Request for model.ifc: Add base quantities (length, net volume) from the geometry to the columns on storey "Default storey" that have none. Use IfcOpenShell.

First a look at what the model holds.

```python
import ifcopenshell
import ifcopenshell.util.element
import ifcopenshell.util.unit

model = ifcopenshell.open("model.ifc")
print(model.schema)
for unit_type in ("LENGTHUNIT", "AREAUNIT", "VOLUMEUNIT"):
    print(unit_type, ifcopenshell.util.unit.calculate_unit_scale(model, unit_type))
storey = next(s for s in model.by_type("IfcBuildingStorey") if s.Name == "Default storey")
columns = [e for e in ifcopenshell.util.element.get_decomposition(storey) if e.is_a("IfcColumn")]
for e in sorted(columns, key=lambda e: e.id()):
    print(e.id(), e.is_a(), e.Name, list(ifcopenshell.util.element.get_psets(e, qtos_only=True)), sep=" | ")
```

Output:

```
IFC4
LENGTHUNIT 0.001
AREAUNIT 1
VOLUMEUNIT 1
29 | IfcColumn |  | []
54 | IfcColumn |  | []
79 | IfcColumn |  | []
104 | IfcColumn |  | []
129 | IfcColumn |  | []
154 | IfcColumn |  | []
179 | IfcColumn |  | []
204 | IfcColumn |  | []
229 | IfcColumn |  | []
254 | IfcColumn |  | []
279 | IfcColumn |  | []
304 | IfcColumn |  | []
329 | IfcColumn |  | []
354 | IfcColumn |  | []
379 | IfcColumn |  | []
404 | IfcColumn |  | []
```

```python
import ifcopenshell
import ifcopenshell.api.pset
import ifcopenshell.geom
import ifcopenshell.util.element
import ifcopenshell.util.shape
import ifcopenshell.util.unit

model = ifcopenshell.open("model.ifc")
unit_scale = ifcopenshell.util.unit.calculate_unit_scale(model)
volume_scale = ifcopenshell.util.unit.calculate_unit_scale(model, "VOLUMEUNIT")
settings = ifcopenshell.geom.settings()

storey = next(s for s in model.by_type("IfcBuildingStorey") if s.Name == "Default storey")
columns = [e for e in ifcopenshell.util.element.get_decomposition(storey) if e.is_a("IfcColumn")]

for e in sorted(columns, key=lambda e: e.id()):
    if ifcopenshell.util.element.get_psets(e, qtos_only=True, should_inherit=False):
        continue
    # Geometry comes back in metres, in the element's own axes.
    shape = ifcopenshell.geom.create_shape(settings, e)
    values = {
        "Length": ifcopenshell.util.shape.get_z(shape.geometry) / unit_scale,
        "NetVolume": ifcopenshell.util.shape.get_volume(shape.geometry) / volume_scale,
    }
    qto = ifcopenshell.api.pset.add_qto(model, product=e, name="Qto_ColumnBaseQuantities")
    ifcopenshell.api.pset.edit_qto(model, qto=qto, properties=values)
    print(e.id(), {k: round(v, 3) for k, v in values.items()})

model.write("model-out.ifc")
```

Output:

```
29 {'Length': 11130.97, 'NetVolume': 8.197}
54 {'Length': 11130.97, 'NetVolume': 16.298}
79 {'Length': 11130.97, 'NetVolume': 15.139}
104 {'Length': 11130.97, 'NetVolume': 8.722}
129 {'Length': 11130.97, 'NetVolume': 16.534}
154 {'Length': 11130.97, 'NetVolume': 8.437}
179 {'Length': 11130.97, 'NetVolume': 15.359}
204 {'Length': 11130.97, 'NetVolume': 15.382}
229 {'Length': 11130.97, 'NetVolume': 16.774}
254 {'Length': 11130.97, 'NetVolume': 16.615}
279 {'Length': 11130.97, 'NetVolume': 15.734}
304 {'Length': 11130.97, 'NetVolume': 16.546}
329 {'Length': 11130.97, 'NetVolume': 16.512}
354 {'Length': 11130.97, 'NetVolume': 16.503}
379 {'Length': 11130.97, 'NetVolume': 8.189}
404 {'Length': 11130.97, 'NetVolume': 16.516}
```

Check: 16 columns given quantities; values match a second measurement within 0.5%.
